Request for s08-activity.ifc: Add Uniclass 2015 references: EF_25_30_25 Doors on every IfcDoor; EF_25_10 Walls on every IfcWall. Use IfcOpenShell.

First a look at what the model holds.

```python
import ifcopenshell

model = ifcopenshell.open("s08-activity.ifc")
print(model.schema)
print("classifications:", [c.Name for c in model.by_type("IfcClassification")])
for ifc_class in ("IfcDoor", "IfcRoof", "IfcStair", "IfcWall", "IfcWindow"):
    print(ifc_class, len(model.by_type(ifc_class)))
```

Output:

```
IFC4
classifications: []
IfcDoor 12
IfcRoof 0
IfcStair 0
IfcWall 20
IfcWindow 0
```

```python
import ifcopenshell
import ifcopenshell.api.classification

model = ifcopenshell.open("s08-activity.ifc")

system = ifcopenshell.api.classification.add_classification(model, classification="Uniclass 2015")

codes = {
    "IfcDoor": ("EF_25_30_25", "Doors"),
    "IfcWall": ("EF_25_10", "Walls"),
}
for ifc_class, (code, name) in codes.items():
    products = model.by_type(ifc_class)
    ifcopenshell.api.classification.add_reference(
        model, products=products, classification=system, identification=code, name=name
    )
    print(code, len(products))

model.write("s08-activity_edited.ifc")
```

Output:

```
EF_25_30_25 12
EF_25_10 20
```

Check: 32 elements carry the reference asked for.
